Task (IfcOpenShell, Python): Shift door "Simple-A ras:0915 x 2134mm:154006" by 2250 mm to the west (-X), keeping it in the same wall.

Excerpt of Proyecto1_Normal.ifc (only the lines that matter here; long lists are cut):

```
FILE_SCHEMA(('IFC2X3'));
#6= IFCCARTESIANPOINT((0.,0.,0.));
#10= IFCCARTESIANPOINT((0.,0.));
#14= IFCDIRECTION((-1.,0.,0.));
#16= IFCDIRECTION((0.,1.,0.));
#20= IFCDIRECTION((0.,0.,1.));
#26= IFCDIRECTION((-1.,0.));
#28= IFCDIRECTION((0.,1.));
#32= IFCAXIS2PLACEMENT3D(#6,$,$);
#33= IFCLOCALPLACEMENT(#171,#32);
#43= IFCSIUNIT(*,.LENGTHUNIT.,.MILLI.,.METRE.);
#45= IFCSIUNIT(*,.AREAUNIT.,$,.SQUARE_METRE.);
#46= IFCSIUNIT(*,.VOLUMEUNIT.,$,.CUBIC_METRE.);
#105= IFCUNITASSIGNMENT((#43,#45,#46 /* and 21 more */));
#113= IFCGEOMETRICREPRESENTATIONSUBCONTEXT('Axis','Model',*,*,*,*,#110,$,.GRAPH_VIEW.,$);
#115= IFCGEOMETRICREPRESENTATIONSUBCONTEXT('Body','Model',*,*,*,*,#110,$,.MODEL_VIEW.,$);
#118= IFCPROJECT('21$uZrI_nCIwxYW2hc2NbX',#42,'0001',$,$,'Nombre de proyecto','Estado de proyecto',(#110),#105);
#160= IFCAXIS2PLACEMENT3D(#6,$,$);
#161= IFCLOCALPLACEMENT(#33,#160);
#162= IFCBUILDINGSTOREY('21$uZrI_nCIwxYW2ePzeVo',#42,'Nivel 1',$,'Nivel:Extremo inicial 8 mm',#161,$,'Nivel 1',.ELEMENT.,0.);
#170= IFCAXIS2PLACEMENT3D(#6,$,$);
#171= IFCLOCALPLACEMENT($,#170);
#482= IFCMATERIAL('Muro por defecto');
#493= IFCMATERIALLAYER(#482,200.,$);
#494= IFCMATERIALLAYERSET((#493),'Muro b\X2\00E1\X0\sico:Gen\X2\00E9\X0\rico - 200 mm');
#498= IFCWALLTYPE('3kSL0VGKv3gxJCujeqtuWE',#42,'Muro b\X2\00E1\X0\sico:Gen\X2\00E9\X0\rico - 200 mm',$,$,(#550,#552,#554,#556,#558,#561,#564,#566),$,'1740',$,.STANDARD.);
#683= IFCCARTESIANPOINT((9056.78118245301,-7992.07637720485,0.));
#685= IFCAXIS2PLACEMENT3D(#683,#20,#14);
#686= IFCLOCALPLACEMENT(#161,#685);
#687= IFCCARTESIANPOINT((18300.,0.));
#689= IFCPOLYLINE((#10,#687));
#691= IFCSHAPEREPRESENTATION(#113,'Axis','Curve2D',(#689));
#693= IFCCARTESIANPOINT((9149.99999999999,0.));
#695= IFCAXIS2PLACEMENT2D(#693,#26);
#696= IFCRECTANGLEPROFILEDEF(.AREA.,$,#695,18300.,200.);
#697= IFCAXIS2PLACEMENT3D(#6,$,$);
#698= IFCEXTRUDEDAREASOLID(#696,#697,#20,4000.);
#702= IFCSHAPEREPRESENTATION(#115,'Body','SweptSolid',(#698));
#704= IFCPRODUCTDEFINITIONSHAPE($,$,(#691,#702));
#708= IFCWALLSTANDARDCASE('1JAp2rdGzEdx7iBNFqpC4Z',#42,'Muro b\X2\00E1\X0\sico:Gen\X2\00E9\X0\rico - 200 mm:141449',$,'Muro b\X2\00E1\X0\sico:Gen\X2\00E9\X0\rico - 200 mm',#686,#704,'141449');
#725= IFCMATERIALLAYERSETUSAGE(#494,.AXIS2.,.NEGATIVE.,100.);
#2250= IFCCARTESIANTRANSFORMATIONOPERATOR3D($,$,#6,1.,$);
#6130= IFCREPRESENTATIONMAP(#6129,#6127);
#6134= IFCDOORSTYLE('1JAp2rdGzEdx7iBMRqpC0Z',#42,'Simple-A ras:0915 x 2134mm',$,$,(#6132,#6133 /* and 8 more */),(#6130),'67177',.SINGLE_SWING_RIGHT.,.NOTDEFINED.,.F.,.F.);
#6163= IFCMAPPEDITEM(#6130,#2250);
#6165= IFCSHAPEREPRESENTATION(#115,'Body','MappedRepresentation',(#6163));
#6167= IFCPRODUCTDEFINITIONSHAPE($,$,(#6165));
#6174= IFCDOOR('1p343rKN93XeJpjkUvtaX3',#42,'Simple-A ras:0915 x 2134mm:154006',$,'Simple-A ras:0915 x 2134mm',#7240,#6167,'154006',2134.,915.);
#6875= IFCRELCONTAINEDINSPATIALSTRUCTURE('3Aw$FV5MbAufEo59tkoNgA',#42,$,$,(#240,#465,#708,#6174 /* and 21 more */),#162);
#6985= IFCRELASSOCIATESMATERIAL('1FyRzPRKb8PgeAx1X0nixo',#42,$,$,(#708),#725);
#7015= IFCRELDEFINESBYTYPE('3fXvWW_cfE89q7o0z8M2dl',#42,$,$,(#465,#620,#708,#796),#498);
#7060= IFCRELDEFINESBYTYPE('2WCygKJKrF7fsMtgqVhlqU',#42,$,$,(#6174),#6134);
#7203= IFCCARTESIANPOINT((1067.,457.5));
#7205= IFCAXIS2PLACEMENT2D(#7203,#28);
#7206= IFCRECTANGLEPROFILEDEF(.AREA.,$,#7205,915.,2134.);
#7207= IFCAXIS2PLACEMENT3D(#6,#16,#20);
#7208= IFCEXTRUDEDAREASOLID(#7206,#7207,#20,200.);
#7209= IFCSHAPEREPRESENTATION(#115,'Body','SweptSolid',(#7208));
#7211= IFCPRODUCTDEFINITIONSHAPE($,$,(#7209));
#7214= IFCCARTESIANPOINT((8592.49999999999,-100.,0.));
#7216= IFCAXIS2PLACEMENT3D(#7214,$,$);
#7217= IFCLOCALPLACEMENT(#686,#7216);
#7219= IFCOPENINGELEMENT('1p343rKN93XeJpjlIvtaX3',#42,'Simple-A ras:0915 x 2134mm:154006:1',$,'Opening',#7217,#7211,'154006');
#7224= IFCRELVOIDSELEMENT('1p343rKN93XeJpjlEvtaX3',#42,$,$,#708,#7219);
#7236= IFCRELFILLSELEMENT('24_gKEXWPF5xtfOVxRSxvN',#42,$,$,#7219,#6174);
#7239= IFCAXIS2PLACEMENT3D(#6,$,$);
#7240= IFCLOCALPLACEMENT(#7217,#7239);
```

```python
import ifcopenshell
import ifcopenshell.api.geometry
import ifcopenshell.util.placement

model = ifcopenshell.open("Proyecto1_Normal.ifc")

door = model.by_guid("1p343rKN93XeJpjkUvtaX3")
opening = door.FillsVoids[0].RelatingOpeningElement
wall = opening.VoidsElements[0].RelatingBuildingElement

wall_matrix = ifcopenshell.util.placement.get_local_placement(wall.ObjectPlacement)
shift = wall_matrix[:3, 0] * 2250.0
before = ifcopenshell.util.placement.get_local_placement(door.ObjectPlacement)[:3, 3].copy()

# The door is placed relative to its opening, so it follows when the opening moves.
matrix = ifcopenshell.util.placement.get_local_placement(opening.ObjectPlacement)
matrix[:3, 3] += shift
ifcopenshell.api.geometry.edit_object_placement(
    model, product=opening, matrix=matrix, is_si=False, should_transform_children=True
)

after = ifcopenshell.util.placement.get_local_placement(door.ObjectPlacement)[:3, 3]
print("door moved by", (after - before).round(3) + 0.0)

model.write("Proyecto1_Normal_v2.ifc")
```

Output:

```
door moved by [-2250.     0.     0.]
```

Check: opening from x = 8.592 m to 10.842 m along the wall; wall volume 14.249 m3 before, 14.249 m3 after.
